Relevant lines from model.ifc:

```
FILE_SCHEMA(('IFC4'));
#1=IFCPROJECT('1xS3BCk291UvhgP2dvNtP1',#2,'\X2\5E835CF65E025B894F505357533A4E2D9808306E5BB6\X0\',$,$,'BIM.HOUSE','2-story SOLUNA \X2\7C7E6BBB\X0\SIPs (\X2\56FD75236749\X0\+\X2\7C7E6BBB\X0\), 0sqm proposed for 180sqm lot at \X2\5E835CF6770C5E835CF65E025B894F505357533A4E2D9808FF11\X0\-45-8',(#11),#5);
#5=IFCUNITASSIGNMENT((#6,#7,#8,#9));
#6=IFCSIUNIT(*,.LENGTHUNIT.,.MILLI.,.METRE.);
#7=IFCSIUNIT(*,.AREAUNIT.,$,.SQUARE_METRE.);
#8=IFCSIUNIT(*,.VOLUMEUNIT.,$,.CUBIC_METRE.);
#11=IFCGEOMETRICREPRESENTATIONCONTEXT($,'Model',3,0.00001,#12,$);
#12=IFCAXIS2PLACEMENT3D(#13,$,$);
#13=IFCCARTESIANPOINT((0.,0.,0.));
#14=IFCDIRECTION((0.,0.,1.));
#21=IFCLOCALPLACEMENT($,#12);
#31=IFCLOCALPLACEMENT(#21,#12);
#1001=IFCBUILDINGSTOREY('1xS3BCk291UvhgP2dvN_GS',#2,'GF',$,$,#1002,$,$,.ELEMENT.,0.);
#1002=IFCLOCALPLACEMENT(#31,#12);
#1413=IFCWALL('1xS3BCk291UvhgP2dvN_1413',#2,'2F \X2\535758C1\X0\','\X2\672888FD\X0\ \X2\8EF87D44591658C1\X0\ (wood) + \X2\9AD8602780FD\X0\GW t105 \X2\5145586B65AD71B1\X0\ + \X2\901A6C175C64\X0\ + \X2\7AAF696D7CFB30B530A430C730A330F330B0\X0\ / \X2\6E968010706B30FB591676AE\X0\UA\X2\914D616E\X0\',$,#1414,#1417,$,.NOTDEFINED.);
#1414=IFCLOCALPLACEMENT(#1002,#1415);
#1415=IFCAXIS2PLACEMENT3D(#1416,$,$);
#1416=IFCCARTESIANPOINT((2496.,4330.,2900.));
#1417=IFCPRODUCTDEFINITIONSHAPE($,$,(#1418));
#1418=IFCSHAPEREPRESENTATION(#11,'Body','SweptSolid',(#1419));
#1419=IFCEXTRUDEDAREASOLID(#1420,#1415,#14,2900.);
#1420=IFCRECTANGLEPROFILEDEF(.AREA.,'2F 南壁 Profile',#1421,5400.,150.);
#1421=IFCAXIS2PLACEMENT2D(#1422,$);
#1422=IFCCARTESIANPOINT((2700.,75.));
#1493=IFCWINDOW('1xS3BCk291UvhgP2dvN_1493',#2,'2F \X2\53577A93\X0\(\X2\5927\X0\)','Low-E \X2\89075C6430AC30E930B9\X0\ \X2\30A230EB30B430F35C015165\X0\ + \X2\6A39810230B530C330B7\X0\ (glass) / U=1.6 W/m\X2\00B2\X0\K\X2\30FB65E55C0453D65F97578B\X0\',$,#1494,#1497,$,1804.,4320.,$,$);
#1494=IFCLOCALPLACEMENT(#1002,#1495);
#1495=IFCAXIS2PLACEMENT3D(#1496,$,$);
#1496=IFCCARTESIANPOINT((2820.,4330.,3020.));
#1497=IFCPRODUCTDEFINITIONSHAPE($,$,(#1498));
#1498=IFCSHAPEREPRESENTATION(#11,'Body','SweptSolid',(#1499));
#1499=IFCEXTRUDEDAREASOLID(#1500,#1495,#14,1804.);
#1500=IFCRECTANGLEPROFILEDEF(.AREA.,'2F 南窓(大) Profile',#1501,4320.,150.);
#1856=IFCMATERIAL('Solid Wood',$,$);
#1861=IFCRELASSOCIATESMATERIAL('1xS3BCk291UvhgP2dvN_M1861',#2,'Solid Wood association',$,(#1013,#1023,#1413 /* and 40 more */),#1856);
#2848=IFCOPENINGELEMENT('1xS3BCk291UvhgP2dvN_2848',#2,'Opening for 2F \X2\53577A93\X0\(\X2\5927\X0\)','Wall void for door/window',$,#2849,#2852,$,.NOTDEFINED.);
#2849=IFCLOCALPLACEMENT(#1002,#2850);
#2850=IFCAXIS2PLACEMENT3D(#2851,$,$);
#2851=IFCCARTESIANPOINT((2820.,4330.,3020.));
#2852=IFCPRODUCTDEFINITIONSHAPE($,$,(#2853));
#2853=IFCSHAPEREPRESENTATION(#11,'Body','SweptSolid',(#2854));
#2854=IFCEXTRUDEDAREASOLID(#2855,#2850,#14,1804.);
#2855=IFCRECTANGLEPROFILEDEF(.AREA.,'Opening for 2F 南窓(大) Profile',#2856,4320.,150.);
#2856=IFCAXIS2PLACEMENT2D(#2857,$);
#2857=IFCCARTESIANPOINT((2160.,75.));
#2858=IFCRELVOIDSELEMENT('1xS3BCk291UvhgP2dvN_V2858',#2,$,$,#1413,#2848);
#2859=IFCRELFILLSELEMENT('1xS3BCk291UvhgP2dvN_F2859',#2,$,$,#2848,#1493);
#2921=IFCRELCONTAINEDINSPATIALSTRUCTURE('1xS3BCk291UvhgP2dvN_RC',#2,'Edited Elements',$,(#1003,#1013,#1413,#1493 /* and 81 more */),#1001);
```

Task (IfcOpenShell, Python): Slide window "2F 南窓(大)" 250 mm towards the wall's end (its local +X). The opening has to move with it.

```python
import ifcopenshell
import ifcopenshell.api.geometry
import ifcopenshell.util.placement
import ifcopenshell.util.unit

model = ifcopenshell.open("model.ifc")
unit_scale = ifcopenshell.util.unit.calculate_unit_scale(model)

window = model.by_id(1493)
opening = window.FillsVoids[0].RelatingOpeningElement
wall = opening.VoidsElements[0].RelatingBuildingElement

wall_matrix = ifcopenshell.util.placement.get_local_placement(wall.ObjectPlacement)
shift = wall_matrix[:3, 0] * 0.25 / unit_scale
before = ifcopenshell.util.placement.get_local_placement(window.ObjectPlacement)[:3, 3].copy()

# The window is not placed relative to its opening, so move both.
for product in (opening, window):
    matrix = ifcopenshell.util.placement.get_local_placement(product.ObjectPlacement)
    matrix[:3, 3] += shift
    ifcopenshell.api.geometry.edit_object_placement(model, product=product, matrix=matrix, is_si=False)

after = ifcopenshell.util.placement.get_local_placement(window.ObjectPlacement)[:3, 3]
print("window moved by", (after - before).round(3) + 0.0)

model.write("model_rev.ifc")
```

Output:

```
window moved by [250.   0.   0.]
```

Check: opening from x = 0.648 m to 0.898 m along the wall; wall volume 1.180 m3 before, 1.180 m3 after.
